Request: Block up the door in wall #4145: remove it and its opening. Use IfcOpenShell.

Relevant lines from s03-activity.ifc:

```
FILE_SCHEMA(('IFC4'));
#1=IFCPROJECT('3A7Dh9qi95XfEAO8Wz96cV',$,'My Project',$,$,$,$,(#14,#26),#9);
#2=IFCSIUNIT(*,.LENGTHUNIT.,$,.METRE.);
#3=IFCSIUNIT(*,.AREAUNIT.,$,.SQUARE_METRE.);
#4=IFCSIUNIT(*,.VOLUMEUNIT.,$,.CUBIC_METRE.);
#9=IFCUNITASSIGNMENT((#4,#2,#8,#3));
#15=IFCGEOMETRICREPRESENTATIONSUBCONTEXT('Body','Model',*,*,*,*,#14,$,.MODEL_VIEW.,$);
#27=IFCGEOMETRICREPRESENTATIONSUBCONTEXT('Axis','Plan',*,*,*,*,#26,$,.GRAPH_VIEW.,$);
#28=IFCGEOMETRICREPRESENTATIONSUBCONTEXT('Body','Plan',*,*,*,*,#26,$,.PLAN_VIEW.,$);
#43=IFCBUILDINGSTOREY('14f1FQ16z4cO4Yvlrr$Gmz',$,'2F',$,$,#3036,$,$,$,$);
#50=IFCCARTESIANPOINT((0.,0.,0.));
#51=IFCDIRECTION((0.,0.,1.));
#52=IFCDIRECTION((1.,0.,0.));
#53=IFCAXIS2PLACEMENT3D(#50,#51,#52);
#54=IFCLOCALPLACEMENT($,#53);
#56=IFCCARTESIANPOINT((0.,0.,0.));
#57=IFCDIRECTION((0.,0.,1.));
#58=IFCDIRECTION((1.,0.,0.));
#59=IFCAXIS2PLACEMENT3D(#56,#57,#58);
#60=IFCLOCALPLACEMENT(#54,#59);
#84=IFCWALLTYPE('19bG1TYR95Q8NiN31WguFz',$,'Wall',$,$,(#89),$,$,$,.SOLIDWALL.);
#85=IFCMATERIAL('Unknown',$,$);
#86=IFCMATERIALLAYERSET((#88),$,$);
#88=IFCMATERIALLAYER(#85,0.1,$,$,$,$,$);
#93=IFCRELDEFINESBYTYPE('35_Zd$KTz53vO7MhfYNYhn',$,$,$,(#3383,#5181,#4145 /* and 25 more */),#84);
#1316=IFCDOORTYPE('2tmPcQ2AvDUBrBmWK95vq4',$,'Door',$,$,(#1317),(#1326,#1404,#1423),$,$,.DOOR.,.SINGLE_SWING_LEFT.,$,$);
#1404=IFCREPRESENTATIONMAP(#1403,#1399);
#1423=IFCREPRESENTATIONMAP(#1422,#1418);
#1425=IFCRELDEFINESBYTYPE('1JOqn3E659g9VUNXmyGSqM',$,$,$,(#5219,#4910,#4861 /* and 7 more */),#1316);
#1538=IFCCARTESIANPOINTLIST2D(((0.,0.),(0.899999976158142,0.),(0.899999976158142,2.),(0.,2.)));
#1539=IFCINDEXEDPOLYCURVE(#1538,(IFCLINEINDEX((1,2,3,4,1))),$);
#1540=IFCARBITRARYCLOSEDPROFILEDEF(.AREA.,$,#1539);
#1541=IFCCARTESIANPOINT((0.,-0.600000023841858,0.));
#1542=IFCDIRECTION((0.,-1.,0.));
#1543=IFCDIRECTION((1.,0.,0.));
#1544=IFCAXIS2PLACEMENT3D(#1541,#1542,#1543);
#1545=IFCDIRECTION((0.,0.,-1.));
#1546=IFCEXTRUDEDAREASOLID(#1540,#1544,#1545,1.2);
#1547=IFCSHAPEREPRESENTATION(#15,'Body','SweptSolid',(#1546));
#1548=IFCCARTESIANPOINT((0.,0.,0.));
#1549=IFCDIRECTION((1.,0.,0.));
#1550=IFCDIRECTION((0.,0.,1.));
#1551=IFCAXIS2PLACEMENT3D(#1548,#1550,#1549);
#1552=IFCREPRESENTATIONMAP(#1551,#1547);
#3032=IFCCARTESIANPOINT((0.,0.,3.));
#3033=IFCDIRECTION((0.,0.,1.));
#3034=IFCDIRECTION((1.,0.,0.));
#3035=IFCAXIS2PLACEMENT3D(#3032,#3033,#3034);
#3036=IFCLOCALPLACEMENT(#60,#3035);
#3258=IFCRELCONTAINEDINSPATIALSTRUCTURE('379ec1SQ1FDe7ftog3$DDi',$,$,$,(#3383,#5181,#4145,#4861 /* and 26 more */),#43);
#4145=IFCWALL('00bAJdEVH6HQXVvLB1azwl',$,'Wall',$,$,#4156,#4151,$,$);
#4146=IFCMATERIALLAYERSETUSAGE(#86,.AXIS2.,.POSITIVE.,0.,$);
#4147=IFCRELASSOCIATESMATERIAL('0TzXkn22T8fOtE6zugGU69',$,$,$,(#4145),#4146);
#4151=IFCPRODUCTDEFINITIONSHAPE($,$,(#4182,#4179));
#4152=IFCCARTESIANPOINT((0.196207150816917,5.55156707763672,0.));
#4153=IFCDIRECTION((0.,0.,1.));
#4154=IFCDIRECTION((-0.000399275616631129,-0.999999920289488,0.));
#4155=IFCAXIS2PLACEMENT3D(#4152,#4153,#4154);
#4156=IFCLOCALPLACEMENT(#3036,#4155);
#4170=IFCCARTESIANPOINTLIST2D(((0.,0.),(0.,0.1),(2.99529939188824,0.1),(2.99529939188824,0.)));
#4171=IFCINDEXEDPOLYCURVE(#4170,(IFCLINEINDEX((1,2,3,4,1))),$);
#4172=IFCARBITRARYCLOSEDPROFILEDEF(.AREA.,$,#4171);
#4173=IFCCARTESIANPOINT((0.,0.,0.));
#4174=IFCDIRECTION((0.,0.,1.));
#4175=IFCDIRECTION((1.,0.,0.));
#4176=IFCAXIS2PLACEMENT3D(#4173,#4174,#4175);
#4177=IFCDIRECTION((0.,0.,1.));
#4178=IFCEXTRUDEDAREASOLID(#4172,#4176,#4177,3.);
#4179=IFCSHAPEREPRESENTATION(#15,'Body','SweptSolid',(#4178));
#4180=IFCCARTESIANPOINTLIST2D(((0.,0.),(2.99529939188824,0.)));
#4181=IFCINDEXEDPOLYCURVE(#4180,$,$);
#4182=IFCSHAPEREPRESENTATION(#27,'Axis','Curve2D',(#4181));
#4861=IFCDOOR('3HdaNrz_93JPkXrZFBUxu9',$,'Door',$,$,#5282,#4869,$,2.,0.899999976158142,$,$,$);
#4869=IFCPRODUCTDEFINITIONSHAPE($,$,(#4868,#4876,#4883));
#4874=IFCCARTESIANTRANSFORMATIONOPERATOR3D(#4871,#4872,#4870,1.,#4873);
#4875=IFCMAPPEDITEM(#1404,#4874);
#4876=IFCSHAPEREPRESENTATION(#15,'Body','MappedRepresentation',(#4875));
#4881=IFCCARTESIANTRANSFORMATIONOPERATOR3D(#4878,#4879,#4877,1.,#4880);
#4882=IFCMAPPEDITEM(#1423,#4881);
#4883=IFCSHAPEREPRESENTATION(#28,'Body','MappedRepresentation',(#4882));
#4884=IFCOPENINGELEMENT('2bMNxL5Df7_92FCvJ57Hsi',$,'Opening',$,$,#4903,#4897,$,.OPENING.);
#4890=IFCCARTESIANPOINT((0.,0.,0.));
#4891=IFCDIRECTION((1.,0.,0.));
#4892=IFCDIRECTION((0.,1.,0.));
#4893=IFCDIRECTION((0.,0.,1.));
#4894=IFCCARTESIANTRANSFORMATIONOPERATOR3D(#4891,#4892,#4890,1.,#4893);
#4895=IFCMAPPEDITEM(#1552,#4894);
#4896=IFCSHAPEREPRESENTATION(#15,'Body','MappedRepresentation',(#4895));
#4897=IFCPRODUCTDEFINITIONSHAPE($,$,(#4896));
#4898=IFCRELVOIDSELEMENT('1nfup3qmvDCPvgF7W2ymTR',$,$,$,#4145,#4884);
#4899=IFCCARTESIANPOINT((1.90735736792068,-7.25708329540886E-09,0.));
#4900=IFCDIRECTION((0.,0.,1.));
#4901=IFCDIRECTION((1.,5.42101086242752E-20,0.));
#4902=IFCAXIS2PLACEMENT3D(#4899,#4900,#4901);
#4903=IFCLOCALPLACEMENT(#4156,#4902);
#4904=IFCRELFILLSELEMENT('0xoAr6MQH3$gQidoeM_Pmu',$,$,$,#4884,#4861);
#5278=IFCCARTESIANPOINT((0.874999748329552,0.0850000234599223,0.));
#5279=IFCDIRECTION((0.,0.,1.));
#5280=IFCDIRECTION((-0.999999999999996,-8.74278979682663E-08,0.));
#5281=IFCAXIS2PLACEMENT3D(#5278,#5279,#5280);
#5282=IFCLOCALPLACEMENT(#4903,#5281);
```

```python
import ifcopenshell
import ifcopenshell.api.feature
import ifcopenshell.api.root
import ifcopenshell.geom
import ifcopenshell.util.shape

model = ifcopenshell.open("s03-activity.ifc")
settings = ifcopenshell.geom.settings()


def volume(element):
    """Net volume in cubic metres, openings subtracted."""
    shape = ifcopenshell.geom.create_shape(settings, element)
    return ifcopenshell.util.shape.get_volume(shape.geometry)


door = model.by_id(4861)
opening = door.FillsVoids[0].RelatingOpeningElement
wall = opening.VoidsElements[0].RelatingBuildingElement
before = volume(wall)

ifcopenshell.api.root.remove_product(model, product=door)
ifcopenshell.api.feature.remove_feature(model, feature=opening)

after = volume(wall)

print(f"wall volume {before:.3f} -> {after:.3f} m3")

model.write("s03-activity_rev.ifc")
```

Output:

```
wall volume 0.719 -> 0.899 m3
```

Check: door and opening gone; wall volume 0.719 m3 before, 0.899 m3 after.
